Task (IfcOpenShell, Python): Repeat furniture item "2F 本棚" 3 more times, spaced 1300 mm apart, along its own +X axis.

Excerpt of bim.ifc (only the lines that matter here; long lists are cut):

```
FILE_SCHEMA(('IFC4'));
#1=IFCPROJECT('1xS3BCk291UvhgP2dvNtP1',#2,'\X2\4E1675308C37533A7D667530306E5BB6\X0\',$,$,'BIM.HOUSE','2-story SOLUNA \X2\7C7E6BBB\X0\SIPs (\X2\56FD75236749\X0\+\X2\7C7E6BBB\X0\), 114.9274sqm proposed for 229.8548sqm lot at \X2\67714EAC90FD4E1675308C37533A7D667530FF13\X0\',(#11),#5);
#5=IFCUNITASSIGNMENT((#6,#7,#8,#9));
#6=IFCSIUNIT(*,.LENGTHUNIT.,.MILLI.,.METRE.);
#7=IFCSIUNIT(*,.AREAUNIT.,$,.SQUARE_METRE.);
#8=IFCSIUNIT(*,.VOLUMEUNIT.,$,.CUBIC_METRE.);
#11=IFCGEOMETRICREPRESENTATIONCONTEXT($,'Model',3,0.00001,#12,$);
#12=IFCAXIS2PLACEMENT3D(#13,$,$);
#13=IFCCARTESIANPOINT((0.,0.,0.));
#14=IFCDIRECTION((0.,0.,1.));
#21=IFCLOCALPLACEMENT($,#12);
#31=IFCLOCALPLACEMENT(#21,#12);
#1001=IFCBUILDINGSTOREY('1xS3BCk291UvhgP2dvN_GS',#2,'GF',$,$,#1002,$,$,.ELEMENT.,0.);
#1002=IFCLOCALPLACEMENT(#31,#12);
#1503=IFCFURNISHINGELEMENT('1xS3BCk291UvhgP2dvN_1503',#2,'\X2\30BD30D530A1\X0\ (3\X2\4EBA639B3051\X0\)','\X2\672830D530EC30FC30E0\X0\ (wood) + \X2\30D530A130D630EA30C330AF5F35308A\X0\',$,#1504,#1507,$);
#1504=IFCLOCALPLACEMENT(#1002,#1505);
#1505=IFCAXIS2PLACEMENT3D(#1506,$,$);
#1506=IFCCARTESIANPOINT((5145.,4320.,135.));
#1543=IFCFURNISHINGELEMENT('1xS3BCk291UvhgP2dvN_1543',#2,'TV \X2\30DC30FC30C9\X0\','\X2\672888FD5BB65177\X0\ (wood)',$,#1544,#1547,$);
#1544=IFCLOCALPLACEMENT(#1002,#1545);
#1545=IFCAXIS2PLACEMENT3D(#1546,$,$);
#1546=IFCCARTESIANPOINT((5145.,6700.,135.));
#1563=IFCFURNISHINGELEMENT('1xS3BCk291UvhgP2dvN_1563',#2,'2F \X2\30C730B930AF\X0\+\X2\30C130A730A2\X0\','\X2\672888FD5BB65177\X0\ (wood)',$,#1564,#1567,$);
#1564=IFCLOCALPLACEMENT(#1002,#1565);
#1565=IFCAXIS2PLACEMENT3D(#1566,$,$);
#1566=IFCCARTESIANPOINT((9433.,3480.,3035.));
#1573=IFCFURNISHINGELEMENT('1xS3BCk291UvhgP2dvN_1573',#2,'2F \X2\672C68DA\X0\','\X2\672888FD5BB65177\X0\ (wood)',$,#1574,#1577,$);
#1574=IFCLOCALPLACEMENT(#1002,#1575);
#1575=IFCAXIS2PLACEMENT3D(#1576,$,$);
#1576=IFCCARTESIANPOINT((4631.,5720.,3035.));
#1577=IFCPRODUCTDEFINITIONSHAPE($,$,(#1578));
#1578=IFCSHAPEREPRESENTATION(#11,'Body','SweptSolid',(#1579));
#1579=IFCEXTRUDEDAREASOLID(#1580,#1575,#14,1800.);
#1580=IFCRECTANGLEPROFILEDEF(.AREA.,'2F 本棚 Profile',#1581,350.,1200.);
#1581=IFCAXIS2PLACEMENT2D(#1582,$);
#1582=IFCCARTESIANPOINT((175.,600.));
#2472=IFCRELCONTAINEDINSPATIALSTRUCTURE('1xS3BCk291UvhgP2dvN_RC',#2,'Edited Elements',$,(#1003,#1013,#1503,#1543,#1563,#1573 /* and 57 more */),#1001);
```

```python
import ifcopenshell
import ifcopenshell.api.geometry
import ifcopenshell.api.root
import ifcopenshell.util.element
import ifcopenshell.util.placement

model = ifcopenshell.open("bim.ifc")


def reuse_history(source, copy):
    """copy_class also copies each property set's owner history, people and application; keep the originals."""
    for rel in copy.IsDefinedBy:
        if rel.is_a("IfcRelDefinesByProperties") and (history := rel.RelatingPropertyDefinition.OwnerHistory):
            rel.RelatingPropertyDefinition.OwnerHistory = source.OwnerHistory
            ifcopenshell.util.element.remove_deep2(model, history)


source = model.by_guid("1xS3BCk291UvhgP2dvN_1573")
base = ifcopenshell.util.placement.get_local_placement(source.ObjectPlacement)
step = base[:3, 0] * 1300.0

for i in range(1, 4):
    copy = ifcopenshell.api.root.copy_class(model, product=source)
    copy.Representation = ifcopenshell.util.element.copy_deep(
        model, source.Representation, exclude=["IfcGeometricRepresentationContext", "IfcRepresentationMap"]
    )
    reuse_history(source, copy)
    matrix = base.copy()
    matrix[:3, 3] += i * step
    print("added at", matrix[:3, 3].round(3) + 0.0)
    ifcopenshell.api.geometry.edit_object_placement(model, product=copy, matrix=matrix, is_si=False)

model.write("bim_rev.ifc")
```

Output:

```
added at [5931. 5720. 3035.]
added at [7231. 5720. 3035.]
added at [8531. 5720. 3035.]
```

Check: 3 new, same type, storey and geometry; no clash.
